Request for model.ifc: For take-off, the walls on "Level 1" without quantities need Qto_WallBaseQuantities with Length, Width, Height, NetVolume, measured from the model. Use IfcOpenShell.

First a look at what the model holds.

```python
import ifcopenshell
import ifcopenshell.util.element
import ifcopenshell.util.unit

model = ifcopenshell.open("model.ifc")
print(model.schema)
for unit_type in ("LENGTHUNIT", "AREAUNIT", "VOLUMEUNIT"):
    print(unit_type, ifcopenshell.util.unit.calculate_unit_scale(model, unit_type))
storey = next(s for s in model.by_type("IfcBuildingStorey") if s.Name == "Level 1")
walls = [e for e in ifcopenshell.util.element.get_decomposition(storey) if e.is_a("IfcWall")]
for e in sorted(walls, key=lambda e: e.id()):
    print(e.id(), e.is_a(), e.Name, list(ifcopenshell.util.element.get_psets(e, qtos_only=True)), sep=" | ")
```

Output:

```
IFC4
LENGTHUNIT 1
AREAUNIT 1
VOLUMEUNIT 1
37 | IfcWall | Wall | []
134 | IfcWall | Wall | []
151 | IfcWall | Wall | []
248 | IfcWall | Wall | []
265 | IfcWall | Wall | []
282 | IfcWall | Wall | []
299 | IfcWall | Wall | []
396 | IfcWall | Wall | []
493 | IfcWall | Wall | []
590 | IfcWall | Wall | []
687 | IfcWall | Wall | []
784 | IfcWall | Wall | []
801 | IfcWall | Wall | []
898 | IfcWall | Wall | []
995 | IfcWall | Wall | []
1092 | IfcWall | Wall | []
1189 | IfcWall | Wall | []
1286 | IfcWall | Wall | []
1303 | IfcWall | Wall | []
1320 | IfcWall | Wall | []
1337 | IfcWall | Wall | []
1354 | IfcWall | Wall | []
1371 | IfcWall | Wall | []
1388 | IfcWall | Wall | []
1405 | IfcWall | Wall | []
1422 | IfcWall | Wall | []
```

```python
import ifcopenshell
import ifcopenshell.api.pset
import ifcopenshell.geom
import ifcopenshell.util.element
import ifcopenshell.util.shape
import ifcopenshell.util.unit

model = ifcopenshell.open("model.ifc")
unit_scale = ifcopenshell.util.unit.calculate_unit_scale(model)
volume_scale = ifcopenshell.util.unit.calculate_unit_scale(model, "VOLUMEUNIT")
settings = ifcopenshell.geom.settings()

storey = next(s for s in model.by_type("IfcBuildingStorey") if s.Name == "Level 1")
walls = [e for e in ifcopenshell.util.element.get_decomposition(storey) if e.is_a("IfcWall")]

for e in sorted(walls, key=lambda e: e.id()):
    if ifcopenshell.util.element.get_psets(e, qtos_only=True, should_inherit=False):
        continue
    # Geometry comes back in metres, in the element's own axes.
    shape = ifcopenshell.geom.create_shape(settings, e)
    values = {
        "Length": ifcopenshell.util.shape.get_x(shape.geometry) / unit_scale,
        "Width": ifcopenshell.util.shape.get_y(shape.geometry) / unit_scale,
        "Height": ifcopenshell.util.shape.get_z(shape.geometry) / unit_scale,
        "NetVolume": ifcopenshell.util.shape.get_volume(shape.geometry) / volume_scale,
    }
    qto = ifcopenshell.api.pset.add_qto(model, product=e, name="Qto_WallBaseQuantities")
    ifcopenshell.api.pset.edit_qto(model, qto=qto, properties=values)
    print(e.id(), {k: round(v, 3) for k, v in values.items()})

model.write("model_v2.ifc")
```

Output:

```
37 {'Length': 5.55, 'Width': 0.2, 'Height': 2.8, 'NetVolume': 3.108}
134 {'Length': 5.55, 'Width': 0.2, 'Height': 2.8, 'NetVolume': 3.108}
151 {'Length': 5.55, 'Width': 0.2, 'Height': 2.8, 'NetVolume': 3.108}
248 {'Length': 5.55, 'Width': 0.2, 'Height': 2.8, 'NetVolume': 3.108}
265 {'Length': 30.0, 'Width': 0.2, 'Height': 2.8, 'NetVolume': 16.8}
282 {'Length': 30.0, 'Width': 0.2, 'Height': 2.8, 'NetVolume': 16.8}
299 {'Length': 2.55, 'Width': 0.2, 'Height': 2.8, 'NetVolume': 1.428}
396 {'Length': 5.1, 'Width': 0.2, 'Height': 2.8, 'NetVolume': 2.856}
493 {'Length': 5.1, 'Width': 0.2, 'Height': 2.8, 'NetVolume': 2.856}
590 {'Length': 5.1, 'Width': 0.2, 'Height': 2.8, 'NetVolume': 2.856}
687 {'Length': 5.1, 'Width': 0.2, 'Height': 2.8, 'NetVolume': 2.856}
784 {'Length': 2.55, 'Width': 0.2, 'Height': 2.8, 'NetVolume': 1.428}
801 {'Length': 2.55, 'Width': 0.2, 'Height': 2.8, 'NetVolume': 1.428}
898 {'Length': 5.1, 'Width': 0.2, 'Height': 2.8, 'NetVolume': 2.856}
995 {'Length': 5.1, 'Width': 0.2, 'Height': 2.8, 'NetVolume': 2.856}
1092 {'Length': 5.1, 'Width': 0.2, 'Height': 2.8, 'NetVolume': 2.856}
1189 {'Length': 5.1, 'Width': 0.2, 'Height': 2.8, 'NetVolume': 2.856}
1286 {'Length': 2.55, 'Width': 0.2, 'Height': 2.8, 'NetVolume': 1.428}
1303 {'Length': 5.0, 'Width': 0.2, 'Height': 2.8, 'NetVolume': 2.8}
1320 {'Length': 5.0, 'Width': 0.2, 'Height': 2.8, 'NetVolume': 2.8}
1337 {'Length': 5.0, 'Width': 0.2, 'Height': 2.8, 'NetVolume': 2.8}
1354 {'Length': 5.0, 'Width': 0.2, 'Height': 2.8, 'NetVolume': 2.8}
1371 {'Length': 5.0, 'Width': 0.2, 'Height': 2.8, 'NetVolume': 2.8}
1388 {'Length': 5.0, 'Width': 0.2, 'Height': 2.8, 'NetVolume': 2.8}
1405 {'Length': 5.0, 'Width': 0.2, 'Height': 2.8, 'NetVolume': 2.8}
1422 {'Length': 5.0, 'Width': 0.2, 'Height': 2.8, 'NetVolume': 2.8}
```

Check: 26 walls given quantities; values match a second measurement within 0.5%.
